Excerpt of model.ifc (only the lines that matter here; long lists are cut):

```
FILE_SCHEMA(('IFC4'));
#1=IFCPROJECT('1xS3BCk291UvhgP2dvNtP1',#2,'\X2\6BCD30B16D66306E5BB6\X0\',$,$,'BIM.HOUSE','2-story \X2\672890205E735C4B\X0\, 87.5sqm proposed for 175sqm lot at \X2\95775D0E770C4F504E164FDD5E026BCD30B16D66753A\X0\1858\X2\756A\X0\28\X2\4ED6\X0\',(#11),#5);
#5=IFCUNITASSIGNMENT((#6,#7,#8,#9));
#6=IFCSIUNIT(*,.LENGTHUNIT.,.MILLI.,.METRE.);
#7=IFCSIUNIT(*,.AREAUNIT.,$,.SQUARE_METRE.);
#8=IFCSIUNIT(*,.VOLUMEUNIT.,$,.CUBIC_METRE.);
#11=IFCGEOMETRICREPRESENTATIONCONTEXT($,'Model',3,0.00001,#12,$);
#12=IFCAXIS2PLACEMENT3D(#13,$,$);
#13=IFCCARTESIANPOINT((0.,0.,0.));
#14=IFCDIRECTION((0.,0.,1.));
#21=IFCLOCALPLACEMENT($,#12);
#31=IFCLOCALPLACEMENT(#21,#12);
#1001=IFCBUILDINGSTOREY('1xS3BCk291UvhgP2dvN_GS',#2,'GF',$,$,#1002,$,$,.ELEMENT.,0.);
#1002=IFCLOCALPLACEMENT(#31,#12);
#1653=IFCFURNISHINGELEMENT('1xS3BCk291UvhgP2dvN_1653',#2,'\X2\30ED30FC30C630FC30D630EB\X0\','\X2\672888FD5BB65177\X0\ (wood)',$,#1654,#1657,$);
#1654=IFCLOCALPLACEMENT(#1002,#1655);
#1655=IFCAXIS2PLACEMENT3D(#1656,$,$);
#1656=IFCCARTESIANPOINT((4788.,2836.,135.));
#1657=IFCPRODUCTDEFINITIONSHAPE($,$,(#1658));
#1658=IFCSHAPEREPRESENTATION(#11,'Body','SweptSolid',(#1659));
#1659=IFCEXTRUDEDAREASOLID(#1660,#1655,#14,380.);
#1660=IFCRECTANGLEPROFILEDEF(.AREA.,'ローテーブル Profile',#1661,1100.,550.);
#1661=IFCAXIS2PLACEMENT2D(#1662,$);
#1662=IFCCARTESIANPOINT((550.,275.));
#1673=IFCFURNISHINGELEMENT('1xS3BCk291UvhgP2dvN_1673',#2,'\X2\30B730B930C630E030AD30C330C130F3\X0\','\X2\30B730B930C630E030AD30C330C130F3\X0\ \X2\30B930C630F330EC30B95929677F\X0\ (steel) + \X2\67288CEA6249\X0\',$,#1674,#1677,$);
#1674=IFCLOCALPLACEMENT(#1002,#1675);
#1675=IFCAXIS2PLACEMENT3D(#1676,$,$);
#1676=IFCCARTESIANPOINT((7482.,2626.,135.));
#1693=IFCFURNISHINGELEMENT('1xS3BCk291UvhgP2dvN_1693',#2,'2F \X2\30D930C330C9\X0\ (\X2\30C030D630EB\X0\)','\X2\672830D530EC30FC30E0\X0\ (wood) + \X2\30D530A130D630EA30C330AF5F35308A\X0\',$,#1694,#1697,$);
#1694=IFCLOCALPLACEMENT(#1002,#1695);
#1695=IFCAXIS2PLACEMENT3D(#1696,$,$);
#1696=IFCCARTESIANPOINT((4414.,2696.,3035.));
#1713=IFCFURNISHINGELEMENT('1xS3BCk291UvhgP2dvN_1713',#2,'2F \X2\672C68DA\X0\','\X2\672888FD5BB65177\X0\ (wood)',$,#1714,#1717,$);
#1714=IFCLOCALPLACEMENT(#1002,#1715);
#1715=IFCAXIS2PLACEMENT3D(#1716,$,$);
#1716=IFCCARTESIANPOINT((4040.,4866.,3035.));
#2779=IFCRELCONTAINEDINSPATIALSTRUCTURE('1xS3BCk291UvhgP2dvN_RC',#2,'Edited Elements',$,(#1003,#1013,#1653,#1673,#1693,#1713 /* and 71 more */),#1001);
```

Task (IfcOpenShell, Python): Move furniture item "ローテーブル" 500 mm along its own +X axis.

```python
import ifcopenshell
import ifcopenshell.api.geometry
import ifcopenshell.util.placement
import ifcopenshell.util.unit

model = ifcopenshell.open("model.ifc")
unit_scale = ifcopenshell.util.unit.calculate_unit_scale(model)

item = model.by_id(1653)
matrix = ifcopenshell.util.placement.get_local_placement(item.ObjectPlacement)
matrix[:3, 3] += matrix[:3, 0] * 0.5 / unit_scale
ifcopenshell.api.geometry.edit_object_placement(model, product=item, matrix=matrix, is_si=False)

print(ifcopenshell.util.placement.get_local_placement(item.ObjectPlacement).round(3) + 0.0)

model.write("model-out.ifc")
```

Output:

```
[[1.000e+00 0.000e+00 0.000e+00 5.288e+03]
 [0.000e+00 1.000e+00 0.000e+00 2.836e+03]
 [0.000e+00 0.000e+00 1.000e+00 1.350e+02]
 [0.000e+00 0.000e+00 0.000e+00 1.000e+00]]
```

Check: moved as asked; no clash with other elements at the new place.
